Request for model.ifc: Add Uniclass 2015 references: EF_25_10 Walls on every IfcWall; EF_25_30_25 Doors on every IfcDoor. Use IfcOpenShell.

First a look at what the model holds.

```python
import ifcopenshell

model = ifcopenshell.open("model.ifc")
print(model.schema)
print("classifications:", [c.Name for c in model.by_type("IfcClassification")])
for ifc_class in ("IfcDoor", "IfcRoof", "IfcStair", "IfcWall", "IfcWindow"):
    print(ifc_class, len(model.by_type(ifc_class)))
```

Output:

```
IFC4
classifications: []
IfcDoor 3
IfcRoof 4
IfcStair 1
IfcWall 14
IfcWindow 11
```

```python
import ifcopenshell
import ifcopenshell.api.classification

model = ifcopenshell.open("model.ifc")

system = ifcopenshell.api.classification.add_classification(model, classification="Uniclass 2015")

codes = {
    "IfcWall": ("EF_25_10", "Walls"),
    "IfcDoor": ("EF_25_30_25", "Doors"),
}
for ifc_class, (code, name) in codes.items():
    products = model.by_type(ifc_class)
    ifcopenshell.api.classification.add_reference(
        model, products=products, classification=system, identification=code, name=name
    )
    print(code, len(products))

model.write("model_v2.ifc")
```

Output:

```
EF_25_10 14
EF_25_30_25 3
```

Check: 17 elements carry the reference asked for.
